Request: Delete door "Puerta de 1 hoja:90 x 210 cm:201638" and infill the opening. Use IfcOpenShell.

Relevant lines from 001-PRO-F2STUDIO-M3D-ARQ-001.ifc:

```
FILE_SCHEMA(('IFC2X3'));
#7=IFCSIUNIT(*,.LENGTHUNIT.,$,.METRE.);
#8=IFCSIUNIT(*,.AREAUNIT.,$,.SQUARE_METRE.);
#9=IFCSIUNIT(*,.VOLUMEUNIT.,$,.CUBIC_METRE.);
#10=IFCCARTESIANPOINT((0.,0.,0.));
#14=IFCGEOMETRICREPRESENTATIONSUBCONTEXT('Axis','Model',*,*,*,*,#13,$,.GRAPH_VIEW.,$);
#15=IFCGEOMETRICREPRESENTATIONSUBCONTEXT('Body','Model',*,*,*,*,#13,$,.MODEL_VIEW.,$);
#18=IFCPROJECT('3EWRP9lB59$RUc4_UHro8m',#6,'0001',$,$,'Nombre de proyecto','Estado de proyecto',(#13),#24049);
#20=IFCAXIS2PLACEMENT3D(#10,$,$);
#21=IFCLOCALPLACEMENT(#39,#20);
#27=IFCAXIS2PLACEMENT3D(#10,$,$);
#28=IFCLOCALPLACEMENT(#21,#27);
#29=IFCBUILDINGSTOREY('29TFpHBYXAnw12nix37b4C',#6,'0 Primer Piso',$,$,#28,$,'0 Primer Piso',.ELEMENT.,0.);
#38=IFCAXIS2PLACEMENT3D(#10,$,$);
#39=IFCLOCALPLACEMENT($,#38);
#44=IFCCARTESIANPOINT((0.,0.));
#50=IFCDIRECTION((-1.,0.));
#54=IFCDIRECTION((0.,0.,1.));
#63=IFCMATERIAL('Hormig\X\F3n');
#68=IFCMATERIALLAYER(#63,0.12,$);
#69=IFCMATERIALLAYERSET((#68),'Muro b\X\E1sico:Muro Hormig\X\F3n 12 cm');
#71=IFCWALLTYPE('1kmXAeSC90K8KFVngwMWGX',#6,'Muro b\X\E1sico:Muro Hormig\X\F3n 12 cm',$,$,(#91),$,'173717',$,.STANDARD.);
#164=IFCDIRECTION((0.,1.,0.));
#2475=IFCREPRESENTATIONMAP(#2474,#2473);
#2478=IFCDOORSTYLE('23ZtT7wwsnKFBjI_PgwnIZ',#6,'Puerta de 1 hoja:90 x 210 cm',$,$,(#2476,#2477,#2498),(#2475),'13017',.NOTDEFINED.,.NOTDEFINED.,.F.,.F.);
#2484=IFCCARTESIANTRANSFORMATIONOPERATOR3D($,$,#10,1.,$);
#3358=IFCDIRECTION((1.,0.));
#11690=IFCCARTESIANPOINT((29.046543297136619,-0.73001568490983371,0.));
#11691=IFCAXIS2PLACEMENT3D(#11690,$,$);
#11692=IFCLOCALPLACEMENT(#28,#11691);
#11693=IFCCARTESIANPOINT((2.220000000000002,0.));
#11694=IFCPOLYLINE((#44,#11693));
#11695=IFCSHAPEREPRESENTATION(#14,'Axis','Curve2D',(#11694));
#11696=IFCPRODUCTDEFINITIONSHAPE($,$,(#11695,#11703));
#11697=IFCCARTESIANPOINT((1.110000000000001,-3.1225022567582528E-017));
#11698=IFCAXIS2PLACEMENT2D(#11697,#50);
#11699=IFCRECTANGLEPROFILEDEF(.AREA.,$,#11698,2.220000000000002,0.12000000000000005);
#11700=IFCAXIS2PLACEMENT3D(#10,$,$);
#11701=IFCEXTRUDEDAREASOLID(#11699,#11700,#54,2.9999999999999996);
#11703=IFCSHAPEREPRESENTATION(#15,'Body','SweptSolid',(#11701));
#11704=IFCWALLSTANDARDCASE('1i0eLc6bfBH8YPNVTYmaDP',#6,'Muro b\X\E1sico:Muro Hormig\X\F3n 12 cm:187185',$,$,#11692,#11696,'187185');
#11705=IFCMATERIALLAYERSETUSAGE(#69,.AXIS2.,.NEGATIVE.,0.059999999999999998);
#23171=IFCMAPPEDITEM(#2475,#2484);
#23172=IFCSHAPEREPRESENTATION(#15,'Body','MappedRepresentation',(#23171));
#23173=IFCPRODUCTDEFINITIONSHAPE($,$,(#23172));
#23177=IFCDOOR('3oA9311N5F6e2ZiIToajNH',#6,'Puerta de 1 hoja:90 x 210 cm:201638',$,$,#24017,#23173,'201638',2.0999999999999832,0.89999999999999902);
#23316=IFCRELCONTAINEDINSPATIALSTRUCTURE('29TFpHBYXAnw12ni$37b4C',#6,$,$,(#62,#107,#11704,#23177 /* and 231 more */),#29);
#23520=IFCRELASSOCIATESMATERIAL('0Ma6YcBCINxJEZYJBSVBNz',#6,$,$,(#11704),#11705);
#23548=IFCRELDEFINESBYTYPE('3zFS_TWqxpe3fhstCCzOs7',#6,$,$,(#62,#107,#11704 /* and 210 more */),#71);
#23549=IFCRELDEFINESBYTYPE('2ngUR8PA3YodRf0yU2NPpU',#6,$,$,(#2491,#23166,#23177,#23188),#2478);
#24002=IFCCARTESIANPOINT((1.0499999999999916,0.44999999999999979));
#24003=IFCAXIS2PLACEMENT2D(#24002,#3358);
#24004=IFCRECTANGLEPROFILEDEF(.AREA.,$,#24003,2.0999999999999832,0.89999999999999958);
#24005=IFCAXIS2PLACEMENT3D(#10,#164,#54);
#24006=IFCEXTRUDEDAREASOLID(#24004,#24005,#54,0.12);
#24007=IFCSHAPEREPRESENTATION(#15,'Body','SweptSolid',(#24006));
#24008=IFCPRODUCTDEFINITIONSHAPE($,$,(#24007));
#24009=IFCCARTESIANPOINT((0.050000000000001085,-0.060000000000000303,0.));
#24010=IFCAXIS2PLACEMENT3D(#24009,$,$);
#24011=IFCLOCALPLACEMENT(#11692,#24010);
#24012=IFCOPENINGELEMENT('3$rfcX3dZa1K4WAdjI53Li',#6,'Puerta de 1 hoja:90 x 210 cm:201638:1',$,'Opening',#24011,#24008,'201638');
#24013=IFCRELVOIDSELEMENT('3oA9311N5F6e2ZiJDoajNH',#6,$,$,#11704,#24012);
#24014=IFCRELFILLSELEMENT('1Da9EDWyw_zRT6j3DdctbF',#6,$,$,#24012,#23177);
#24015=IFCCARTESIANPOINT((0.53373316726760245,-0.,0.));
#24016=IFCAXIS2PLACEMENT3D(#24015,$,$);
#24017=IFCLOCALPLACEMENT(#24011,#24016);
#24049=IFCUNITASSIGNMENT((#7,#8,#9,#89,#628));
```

```python
import ifcopenshell
import ifcopenshell.api.feature
import ifcopenshell.api.root
import ifcopenshell.geom
import ifcopenshell.util.shape

model = ifcopenshell.open("001-PRO-F2STUDIO-M3D-ARQ-001.ifc")
settings = ifcopenshell.geom.settings()


def volume(element):
    """Net volume in cubic metres, openings subtracted."""
    shape = ifcopenshell.geom.create_shape(settings, element)
    return ifcopenshell.util.shape.get_volume(shape.geometry)


door = model.by_guid("3oA9311N5F6e2ZiIToajNH")
opening = door.FillsVoids[0].RelatingOpeningElement
wall = opening.VoidsElements[0].RelatingBuildingElement
before = volume(wall)

ifcopenshell.api.root.remove_product(model, product=door)
ifcopenshell.api.feature.remove_feature(model, feature=opening)

after = volume(wall)

print(f"wall volume {before:.3f} -> {after:.3f} m3")

model.write("001-PRO-F2STUDIO-M3D-ARQ-001-out.ifc")
```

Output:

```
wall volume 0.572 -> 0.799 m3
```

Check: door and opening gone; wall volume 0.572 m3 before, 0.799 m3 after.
